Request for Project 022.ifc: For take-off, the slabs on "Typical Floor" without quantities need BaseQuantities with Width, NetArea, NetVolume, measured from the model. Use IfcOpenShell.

First a look at what the model holds.

```python
import ifcopenshell
import ifcopenshell.util.element
import ifcopenshell.util.unit

model = ifcopenshell.open("Project 022.ifc")
print(model.schema)
for unit_type in ("LENGTHUNIT", "AREAUNIT", "VOLUMEUNIT"):
    print(unit_type, ifcopenshell.util.unit.calculate_unit_scale(model, unit_type))
storey = next(s for s in model.by_type("IfcBuildingStorey") if s.Name == "Typical Floor")
slabs = [e for e in ifcopenshell.util.element.get_decomposition(storey) if e.is_a("IfcSlab")]
for e in sorted(slabs, key=lambda e: e.id()):
    print(e.id(), e.is_a(), e.Name, list(ifcopenshell.util.element.get_psets(e, qtos_only=True)), sep=" | ")
```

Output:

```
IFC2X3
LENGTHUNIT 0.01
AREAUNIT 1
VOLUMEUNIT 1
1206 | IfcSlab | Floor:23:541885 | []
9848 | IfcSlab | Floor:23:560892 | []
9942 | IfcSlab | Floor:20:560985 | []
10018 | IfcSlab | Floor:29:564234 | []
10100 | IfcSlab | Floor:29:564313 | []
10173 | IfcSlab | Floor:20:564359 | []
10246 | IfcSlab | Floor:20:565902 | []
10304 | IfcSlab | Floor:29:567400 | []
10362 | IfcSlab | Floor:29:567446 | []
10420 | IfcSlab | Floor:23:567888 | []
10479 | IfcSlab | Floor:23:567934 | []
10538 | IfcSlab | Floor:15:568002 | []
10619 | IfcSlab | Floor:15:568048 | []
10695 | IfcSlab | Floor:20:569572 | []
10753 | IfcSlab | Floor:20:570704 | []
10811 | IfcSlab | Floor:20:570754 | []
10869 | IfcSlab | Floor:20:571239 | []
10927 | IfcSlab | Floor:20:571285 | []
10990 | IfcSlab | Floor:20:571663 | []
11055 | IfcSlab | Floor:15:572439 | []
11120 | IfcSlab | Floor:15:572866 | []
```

```python
import ifcopenshell
import ifcopenshell.api.pset
import ifcopenshell.geom
import ifcopenshell.util.element
import ifcopenshell.util.shape
import ifcopenshell.util.unit

model = ifcopenshell.open("Project 022.ifc")
unit_scale = ifcopenshell.util.unit.calculate_unit_scale(model)
area_scale = ifcopenshell.util.unit.calculate_unit_scale(model, "AREAUNIT")
volume_scale = ifcopenshell.util.unit.calculate_unit_scale(model, "VOLUMEUNIT")
settings = ifcopenshell.geom.settings()

storey = next(s for s in model.by_type("IfcBuildingStorey") if s.Name == "Typical Floor")
slabs = [e for e in ifcopenshell.util.element.get_decomposition(storey) if e.is_a("IfcSlab")]

for e in sorted(slabs, key=lambda e: e.id()):
    if ifcopenshell.util.element.get_psets(e, qtos_only=True, should_inherit=False):
        continue
    # Geometry comes back in metres, in the element's own axes.
    shape = ifcopenshell.geom.create_shape(settings, e)
    values = {
        "Width": ifcopenshell.util.shape.get_z(shape.geometry) / unit_scale,
        "NetArea": ifcopenshell.util.shape.get_footprint_area(shape.geometry) / area_scale,
        "NetVolume": ifcopenshell.util.shape.get_volume(shape.geometry) / volume_scale,
    }
    qto = ifcopenshell.api.pset.add_qto(model, product=e, name="BaseQuantities")
    ifcopenshell.api.pset.edit_qto(model, qto=qto, properties=values)
    print(e.id(), {k: round(v, 3) for k, v in values.items()})

model.write("Project 022-out.ifc")
```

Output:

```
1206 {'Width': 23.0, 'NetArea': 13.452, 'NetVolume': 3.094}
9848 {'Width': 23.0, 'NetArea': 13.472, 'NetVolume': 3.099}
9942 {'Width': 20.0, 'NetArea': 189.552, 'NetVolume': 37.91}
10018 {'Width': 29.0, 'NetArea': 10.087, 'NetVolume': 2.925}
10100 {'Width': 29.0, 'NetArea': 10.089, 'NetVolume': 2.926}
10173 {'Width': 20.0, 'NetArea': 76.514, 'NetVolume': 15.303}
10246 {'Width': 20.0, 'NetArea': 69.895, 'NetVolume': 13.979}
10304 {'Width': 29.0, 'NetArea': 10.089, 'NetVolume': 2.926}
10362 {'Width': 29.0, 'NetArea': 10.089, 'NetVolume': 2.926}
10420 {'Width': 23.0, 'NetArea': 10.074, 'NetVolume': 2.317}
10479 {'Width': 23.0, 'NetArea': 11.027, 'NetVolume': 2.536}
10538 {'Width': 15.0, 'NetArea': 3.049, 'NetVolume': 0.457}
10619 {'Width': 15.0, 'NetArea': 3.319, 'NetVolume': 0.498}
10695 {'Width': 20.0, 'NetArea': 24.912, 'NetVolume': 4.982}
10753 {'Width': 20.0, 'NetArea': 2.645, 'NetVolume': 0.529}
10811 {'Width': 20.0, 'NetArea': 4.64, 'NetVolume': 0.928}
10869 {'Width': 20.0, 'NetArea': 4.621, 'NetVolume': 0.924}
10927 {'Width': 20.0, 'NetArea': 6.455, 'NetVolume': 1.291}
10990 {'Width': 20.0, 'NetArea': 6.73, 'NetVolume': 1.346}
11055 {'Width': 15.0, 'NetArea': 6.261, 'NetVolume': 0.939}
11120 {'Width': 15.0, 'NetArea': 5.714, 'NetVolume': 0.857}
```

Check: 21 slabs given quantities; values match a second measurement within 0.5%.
